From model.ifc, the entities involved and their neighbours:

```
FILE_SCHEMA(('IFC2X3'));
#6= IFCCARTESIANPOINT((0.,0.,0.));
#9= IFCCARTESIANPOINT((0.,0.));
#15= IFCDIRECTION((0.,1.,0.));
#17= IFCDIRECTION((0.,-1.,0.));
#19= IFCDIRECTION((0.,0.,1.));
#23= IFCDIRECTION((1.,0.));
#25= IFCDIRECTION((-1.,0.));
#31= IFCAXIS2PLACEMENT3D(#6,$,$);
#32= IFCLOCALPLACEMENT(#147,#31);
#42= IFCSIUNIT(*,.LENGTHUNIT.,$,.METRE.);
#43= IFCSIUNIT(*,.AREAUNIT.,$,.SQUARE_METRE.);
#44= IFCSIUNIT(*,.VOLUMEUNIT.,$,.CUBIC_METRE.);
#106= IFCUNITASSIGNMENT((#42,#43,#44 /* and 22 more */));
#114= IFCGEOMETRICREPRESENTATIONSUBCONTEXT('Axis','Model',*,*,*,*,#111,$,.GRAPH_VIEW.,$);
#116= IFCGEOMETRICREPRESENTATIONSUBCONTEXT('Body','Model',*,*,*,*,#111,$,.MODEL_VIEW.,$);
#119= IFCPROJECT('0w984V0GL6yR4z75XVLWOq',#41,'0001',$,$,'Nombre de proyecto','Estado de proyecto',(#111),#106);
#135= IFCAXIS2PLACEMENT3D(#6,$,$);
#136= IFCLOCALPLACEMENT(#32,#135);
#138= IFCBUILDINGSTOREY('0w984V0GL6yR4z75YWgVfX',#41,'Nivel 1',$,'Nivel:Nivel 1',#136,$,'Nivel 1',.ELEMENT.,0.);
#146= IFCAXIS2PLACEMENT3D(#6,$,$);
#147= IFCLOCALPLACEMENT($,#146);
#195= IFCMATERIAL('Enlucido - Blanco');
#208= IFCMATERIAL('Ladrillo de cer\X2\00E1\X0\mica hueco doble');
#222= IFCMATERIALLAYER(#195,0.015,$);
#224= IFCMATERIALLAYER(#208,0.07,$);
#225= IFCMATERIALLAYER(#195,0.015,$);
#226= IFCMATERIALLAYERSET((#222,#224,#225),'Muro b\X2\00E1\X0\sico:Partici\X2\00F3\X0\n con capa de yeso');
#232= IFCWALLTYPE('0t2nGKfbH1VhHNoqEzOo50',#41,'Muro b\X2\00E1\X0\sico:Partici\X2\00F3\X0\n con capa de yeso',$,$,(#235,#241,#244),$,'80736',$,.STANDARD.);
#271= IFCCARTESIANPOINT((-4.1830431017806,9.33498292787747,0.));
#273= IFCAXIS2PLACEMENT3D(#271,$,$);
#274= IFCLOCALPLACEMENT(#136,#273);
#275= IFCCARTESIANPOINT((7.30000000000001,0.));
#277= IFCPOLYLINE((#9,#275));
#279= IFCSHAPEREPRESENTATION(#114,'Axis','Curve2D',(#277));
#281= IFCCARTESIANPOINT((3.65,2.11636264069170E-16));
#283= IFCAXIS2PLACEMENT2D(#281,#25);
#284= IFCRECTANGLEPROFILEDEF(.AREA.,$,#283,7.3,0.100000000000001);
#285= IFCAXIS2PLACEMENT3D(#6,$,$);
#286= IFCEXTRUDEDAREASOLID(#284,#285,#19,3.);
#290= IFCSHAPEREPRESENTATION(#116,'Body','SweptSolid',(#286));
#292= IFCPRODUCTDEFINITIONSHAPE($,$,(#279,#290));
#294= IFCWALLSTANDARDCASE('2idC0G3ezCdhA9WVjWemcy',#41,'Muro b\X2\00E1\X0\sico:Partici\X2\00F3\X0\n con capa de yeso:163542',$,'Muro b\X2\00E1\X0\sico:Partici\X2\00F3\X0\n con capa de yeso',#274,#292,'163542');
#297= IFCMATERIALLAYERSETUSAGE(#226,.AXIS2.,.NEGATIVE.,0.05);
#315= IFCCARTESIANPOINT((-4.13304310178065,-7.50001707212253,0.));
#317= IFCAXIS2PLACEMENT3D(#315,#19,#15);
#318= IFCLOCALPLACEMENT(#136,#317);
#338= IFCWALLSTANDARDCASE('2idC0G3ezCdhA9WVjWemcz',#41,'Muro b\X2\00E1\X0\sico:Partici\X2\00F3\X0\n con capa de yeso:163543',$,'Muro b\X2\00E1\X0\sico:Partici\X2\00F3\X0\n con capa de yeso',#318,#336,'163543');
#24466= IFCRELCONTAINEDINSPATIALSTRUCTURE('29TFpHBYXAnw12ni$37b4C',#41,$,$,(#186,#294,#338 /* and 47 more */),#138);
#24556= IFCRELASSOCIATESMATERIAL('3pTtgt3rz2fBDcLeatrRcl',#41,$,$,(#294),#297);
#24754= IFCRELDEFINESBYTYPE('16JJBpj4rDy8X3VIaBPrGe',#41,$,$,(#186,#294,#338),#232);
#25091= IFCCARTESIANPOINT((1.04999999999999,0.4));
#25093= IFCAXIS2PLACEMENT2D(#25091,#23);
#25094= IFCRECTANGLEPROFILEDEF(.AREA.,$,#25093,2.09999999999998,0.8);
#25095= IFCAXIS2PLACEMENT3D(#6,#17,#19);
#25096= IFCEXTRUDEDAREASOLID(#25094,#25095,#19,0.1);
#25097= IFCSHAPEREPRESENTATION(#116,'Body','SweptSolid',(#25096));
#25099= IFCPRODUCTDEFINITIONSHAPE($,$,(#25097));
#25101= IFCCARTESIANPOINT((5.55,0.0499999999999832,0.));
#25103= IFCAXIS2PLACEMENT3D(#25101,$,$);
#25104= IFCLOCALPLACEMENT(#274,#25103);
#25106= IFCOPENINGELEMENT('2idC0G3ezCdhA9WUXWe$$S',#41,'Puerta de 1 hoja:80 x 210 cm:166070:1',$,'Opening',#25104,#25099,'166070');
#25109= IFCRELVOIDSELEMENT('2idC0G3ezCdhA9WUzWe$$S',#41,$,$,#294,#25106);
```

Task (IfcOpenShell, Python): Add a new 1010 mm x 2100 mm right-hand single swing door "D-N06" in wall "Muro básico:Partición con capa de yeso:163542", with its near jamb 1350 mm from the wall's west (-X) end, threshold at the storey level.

```python
import numpy as np
import ifcopenshell
import ifcopenshell.api.feature
import ifcopenshell.api.geometry
import ifcopenshell.api.root
import ifcopenshell.api.spatial
import ifcopenshell.api.type
import ifcopenshell.geom
import ifcopenshell.util.element
import ifcopenshell.util.placement
import ifcopenshell.util.representation
import ifcopenshell.util.shape
import ifcopenshell.util.unit

model = ifcopenshell.open("model.ifc")
unit_scale = ifcopenshell.util.unit.calculate_unit_scale(model)
settings = ifcopenshell.geom.settings()


def volume(element):
    """Net volume in cubic metres, openings subtracted."""
    shape = ifcopenshell.geom.create_shape(settings, element)
    return ifcopenshell.util.shape.get_volume(shape.geometry)


wall = model.by_guid("2idC0G3ezCdhA9WVjWemcy")
storey = ifcopenshell.util.element.get_container(wall, ifc_class="IfcBuildingStorey")
context = ifcopenshell.util.representation.get_context(model, "Model", "Body", "MODEL_VIEW")
before = volume(wall)

width, height, from_end, sill = 1.01, 2.1, 1.35, 0.0  # metres

# The wall runs along its own X axis, and the end named is its -X end.
wall_shape = ifcopenshell.geom.create_shape(settings, wall)
x, y, z = ifcopenshell.util.shape.get_vertices(wall_shape.geometry).T
start = x.min() + from_end
face, thickness = float(y.min()), float(y.max() - y.min())
wall_matrix = ifcopenshell.util.placement.get_local_placement(wall.ObjectPlacement)
level = ifcopenshell.util.placement.get_local_placement(storey.ObjectPlacement)[2, 3]


def in_wall(x, y):
    """Placement at x, y metres in the wall's axes, at sill height."""
    matrix = wall_matrix.copy()
    matrix[:, 3] = wall_matrix @ np.array([x / unit_scale, y / unit_scale, 0.0, 1.0])
    matrix[2, 3] = level + sill / unit_scale
    return matrix


# Opening: a box that overshoots both wall faces by 50 mm.
opening = ifcopenshell.api.root.create_entity(model, ifc_class="IfcOpeningElement")
box = ifcopenshell.api.geometry.add_wall_representation(
    model, context=context, length=width, height=height, thickness=thickness + 0.1
)
ifcopenshell.api.geometry.assign_representation(model, product=opening, representation=box)
ifcopenshell.api.geometry.edit_object_placement(model, product=opening, matrix=in_wall(start, face - 0.05), is_si=False)
ifcopenshell.api.feature.add_feature(model, feature=opening, element=wall)

door = ifcopenshell.api.root.create_entity(model, ifc_class="IfcDoor", name="D-N06")
door.OverallWidth, door.OverallHeight = width / unit_scale, height / unit_scale
body = ifcopenshell.api.geometry.add_door_representation(
    model,
    context=context,
    overall_width=door.OverallWidth,
    overall_height=door.OverallHeight,
    operation_type="SINGLE_SWING_RIGHT",
    lining_properties={"LiningDepth": thickness / unit_scale, "ThresholdDepth": thickness / unit_scale},
)
ifcopenshell.api.geometry.assign_representation(model, product=door, representation=body)
ifcopenshell.api.spatial.assign_container(model, products=[door], relating_structure=storey)
fills = ifcopenshell.api.feature.add_filling(model, opening=opening, element=door)
fills.OwnerHistory = door.OwnerHistory  # required in IFC2X3

# IFC2X3 keeps the operation on the door style.
style = ifcopenshell.api.root.create_entity(model, ifc_class="IfcDoorStyle", name="D-N06")
style.OperationType, style.ConstructionType = "SINGLE_SWING_RIGHT", "NOTDEFINED"
style.ParameterTakesPrecedence = style.Sizeable = False
ifcopenshell.api.type.assign_type(model, related_objects=[door], relating_type=style)

# The lining spans the wall, so the door starts at the wall face.
ifcopenshell.api.geometry.edit_object_placement(model, product=door, matrix=in_wall(start, face), is_si=False)

after = volume(wall)

print(f"wall volume {before:.3f} -> {after:.3f} m3")

model.write("model_edited.ifc")
```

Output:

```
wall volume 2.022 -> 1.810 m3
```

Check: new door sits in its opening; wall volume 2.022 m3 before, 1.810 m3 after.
